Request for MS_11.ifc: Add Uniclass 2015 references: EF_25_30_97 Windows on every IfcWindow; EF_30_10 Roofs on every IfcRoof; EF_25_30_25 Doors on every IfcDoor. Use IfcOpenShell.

First a look at what the model holds.

```python
import ifcopenshell

model = ifcopenshell.open("MS_11.ifc")
print(model.schema)
print("classifications:", [c.Name for c in model.by_type("IfcClassification")])
for ifc_class in ("IfcDoor", "IfcRoof", "IfcStair", "IfcWall", "IfcWindow"):
    print(ifc_class, len(model.by_type(ifc_class)))
```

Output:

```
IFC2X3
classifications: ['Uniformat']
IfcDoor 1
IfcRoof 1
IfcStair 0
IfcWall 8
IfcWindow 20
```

```python
import ifcopenshell
import ifcopenshell.api.classification

model = ifcopenshell.open("MS_11.ifc")

# IFC2X3 requires Source and Edition and has no link from the project to the system.
system = model.create_entity("IfcClassification", Source="NBS", Edition="2015", Name="Uniclass 2015")

codes = {
    "IfcWindow": ("EF_25_30_97", "Windows"),
    "IfcRoof": ("EF_30_10", "Roofs"),
    "IfcDoor": ("EF_25_30_25", "Doors"),
}
for ifc_class, (code, name) in codes.items():
    products = model.by_type(ifc_class)
    ifcopenshell.api.classification.add_reference(
        model, products=products, classification=system, identification=code, name=name
    )
    print(code, len(products))

model.write("MS_11_updated.ifc")
```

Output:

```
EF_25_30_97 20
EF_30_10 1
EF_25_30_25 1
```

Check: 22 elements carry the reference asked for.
